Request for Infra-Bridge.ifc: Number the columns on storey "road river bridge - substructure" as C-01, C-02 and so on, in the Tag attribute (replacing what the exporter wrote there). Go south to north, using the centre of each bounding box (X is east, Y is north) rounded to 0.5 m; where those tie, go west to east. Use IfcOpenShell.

First a look at what the model holds.

```python
import ifcopenshell
import ifcopenshell.util.element
import ifcopenshell.util.placement

model = ifcopenshell.open("Infra-Bridge.ifc")
print(model.schema)
storey = next(s for s in model.by_type("IfcBuildingStorey") if s.Name == "road river bridge - substructure")
columns = [e for e in ifcopenshell.util.element.get_decomposition(storey) if e.is_a("IfcColumn")]
for e in sorted(columns, key=lambda e: e.id()):
    origin = ifcopenshell.util.placement.get_local_placement(e.ObjectPlacement)[:3, 3]
    print(e.id(), e.Tag, e.Name, origin.round(2) + 0.0, sep=" | ")
```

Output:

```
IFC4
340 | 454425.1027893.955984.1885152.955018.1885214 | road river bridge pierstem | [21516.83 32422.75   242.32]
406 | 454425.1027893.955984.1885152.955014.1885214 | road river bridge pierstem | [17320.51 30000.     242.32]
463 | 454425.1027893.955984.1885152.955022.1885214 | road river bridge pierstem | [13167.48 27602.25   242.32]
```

```python
import ifcopenshell
import ifcopenshell.geom
import ifcopenshell.util.element
import ifcopenshell.util.shape

model = ifcopenshell.open("Infra-Bridge.ifc")
settings = ifcopenshell.geom.settings()
settings.set("use-world-coords", True)


def centre(element):
    shape = ifcopenshell.geom.create_shape(settings, element)
    return ifcopenshell.util.shape.get_bbox_centroid(shape.geometry)


storey = next(s for s in model.by_type("IfcBuildingStorey") if s.Name == "road river bridge - substructure")
columns = [e for e in ifcopenshell.util.element.get_decomposition(storey) if e.is_a("IfcColumn")]

# Insertion points can sit at a corner or the storey origin, so sort by the geometry (in metres).
centres = {e: centre(e) for e in columns}
columns.sort(key=lambda e: (round(centres[e][1] / 0.5), centres[e][0]))

for i, e in enumerate(columns, start=1):
    number = f"C-{i:02d}"
    e.Tag = number
    print(e.id(), number)

model.write("Infra-Bridge_v2.ifc")
```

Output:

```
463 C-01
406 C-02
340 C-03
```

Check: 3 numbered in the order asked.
